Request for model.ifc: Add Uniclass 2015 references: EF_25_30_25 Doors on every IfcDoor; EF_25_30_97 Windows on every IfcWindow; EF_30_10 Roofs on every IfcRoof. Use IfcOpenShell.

First a look at what the model holds.

```python
import ifcopenshell

model = ifcopenshell.open("model.ifc")
print(model.schema)
print("classifications:", [c.Name for c in model.by_type("IfcClassification")])
for ifc_class in ("IfcDoor", "IfcRoof", "IfcStair", "IfcWall", "IfcWindow"):
    print(ifc_class, len(model.by_type(ifc_class)))
```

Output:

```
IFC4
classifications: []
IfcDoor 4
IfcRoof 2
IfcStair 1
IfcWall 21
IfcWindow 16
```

```python
import ifcopenshell
import ifcopenshell.api.classification

model = ifcopenshell.open("model.ifc")

system = ifcopenshell.api.classification.add_classification(model, classification="Uniclass 2015")

codes = {
    "IfcDoor": ("EF_25_30_25", "Doors"),
    "IfcWindow": ("EF_25_30_97", "Windows"),
    "IfcRoof": ("EF_30_10", "Roofs"),
}
for ifc_class, (code, name) in codes.items():
    products = model.by_type(ifc_class)
    ifcopenshell.api.classification.add_reference(
        model, products=products, classification=system, identification=code, name=name
    )
    print(code, len(products))

model.write("model_edited.ifc")
```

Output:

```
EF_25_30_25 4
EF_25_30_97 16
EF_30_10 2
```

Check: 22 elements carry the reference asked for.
